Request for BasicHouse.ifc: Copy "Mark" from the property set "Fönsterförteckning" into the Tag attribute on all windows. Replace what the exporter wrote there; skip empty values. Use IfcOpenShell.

First a look at what the model holds.

```python
import ifcopenshell
import ifcopenshell.util.element

model = ifcopenshell.open("BasicHouse.ifc")
print(model.schema)
windows = model.by_type("IfcWindow")
print(len(windows), "windows")
for e in windows[:8]:
    source = ifcopenshell.util.element.get_pset(e, "Fönsterförteckning", "Mark")
    target = e.Tag
    print(e.id(), repr(source), repr(target), sep=" | ")
```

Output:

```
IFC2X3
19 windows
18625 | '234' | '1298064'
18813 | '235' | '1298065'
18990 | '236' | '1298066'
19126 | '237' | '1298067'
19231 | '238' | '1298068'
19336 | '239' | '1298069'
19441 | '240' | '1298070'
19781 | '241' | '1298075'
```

```python
import ifcopenshell
import ifcopenshell.util.element

model = ifcopenshell.open("BasicHouse.ifc")

count = 0
for e in model.by_type("IfcWindow"):
    value = ifcopenshell.util.element.get_pset(e, "Fönsterförteckning", "Mark")
    current = e.Tag
    if not value or not value.strip() or current == value:
        continue
    e.Tag = value
    count += 1

print(count, "windows updated")

model.write("BasicHouse_updated.ifc")
```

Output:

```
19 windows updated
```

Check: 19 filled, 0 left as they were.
